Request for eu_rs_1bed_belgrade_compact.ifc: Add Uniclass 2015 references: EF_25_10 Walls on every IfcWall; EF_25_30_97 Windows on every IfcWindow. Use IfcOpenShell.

First a look at what the model holds.

```python
import ifcopenshell

model = ifcopenshell.open("eu_rs_1bed_belgrade_compact.ifc")
print(model.schema)
print("classifications:", [c.Name for c in model.by_type("IfcClassification")])
for ifc_class in ("IfcDoor", "IfcRoof", "IfcStair", "IfcWall", "IfcWindow"):
    print(ifc_class, len(model.by_type(ifc_class)))
```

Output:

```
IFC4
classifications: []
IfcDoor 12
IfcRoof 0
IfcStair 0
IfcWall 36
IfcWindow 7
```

```python
import ifcopenshell
import ifcopenshell.api.classification

model = ifcopenshell.open("eu_rs_1bed_belgrade_compact.ifc")

system = ifcopenshell.api.classification.add_classification(model, classification="Uniclass 2015")

codes = {
    "IfcWall": ("EF_25_10", "Walls"),
    "IfcWindow": ("EF_25_30_97", "Windows"),
}
for ifc_class, (code, name) in codes.items():
    products = model.by_type(ifc_class)
    ifcopenshell.api.classification.add_reference(
        model, products=products, classification=system, identification=code, name=name
    )
    print(code, len(products))

model.write("eu_rs_1bed_belgrade_compact_edited.ifc")
```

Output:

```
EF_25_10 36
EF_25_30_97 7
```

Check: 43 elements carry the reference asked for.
